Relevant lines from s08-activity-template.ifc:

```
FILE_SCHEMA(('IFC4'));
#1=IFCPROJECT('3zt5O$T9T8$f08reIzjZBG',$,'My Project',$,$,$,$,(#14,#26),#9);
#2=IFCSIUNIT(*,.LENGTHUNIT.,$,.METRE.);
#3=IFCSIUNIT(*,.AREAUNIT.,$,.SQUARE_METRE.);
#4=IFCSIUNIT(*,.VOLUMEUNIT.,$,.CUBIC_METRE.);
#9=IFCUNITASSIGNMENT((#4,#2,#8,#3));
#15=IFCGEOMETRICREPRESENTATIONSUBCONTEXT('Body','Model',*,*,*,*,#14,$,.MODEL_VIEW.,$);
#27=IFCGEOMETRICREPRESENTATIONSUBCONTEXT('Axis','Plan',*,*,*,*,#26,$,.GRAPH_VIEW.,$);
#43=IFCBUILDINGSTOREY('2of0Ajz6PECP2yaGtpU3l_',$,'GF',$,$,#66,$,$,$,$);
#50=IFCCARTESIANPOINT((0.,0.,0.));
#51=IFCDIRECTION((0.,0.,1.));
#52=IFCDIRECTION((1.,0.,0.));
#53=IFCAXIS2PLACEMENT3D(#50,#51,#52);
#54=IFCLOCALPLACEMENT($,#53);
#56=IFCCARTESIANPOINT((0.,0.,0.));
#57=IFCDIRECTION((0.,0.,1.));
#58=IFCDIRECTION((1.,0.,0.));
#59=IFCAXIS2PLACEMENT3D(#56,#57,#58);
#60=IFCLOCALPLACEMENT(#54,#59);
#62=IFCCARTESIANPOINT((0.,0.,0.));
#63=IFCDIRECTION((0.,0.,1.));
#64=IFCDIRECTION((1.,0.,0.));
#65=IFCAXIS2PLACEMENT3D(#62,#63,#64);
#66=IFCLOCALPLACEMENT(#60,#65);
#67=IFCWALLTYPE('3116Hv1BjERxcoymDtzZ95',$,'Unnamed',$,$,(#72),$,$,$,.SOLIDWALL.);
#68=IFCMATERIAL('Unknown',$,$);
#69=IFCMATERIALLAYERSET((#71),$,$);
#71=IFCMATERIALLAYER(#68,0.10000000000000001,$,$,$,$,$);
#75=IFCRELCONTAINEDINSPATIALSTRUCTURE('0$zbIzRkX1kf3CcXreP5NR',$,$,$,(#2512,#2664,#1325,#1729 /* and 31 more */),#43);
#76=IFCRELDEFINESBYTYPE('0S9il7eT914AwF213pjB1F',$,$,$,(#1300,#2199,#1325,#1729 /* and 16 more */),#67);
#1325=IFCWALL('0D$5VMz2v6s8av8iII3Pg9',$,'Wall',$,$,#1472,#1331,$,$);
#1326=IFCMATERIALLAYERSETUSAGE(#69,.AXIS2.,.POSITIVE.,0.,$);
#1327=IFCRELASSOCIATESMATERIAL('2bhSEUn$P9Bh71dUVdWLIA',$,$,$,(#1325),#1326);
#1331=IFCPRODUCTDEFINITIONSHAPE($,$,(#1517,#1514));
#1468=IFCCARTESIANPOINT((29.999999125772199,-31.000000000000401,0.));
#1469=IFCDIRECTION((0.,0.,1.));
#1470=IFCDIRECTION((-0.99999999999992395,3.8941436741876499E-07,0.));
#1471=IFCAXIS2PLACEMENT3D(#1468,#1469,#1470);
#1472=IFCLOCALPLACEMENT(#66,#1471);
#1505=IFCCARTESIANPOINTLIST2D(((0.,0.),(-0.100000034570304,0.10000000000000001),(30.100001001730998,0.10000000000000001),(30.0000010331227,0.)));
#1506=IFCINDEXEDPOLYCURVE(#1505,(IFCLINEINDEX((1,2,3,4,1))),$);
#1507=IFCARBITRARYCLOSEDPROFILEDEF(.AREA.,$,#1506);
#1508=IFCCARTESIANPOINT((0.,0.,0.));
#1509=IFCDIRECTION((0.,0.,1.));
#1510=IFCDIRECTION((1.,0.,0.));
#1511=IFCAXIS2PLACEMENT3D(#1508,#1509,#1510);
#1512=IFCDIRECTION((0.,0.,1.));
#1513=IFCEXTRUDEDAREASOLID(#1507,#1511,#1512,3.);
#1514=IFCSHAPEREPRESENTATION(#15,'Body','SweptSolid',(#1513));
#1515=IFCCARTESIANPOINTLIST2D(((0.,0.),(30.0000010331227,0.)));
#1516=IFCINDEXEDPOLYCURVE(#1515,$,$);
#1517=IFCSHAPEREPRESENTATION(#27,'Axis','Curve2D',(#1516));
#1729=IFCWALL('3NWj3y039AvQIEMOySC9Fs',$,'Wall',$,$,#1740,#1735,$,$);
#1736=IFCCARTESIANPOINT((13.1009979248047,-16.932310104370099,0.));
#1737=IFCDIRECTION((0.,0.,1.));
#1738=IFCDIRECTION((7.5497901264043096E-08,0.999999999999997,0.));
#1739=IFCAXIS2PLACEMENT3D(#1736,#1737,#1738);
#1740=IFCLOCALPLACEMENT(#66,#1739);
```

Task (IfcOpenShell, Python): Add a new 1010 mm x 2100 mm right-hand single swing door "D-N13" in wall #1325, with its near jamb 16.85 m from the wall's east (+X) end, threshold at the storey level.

```python
import numpy as np
import ifcopenshell
import ifcopenshell.api.feature
import ifcopenshell.api.geometry
import ifcopenshell.api.root
import ifcopenshell.api.spatial
import ifcopenshell.geom
import ifcopenshell.util.element
import ifcopenshell.util.placement
import ifcopenshell.util.representation
import ifcopenshell.util.shape
import ifcopenshell.util.unit

model = ifcopenshell.open("s08-activity-template.ifc")
unit_scale = ifcopenshell.util.unit.calculate_unit_scale(model)
settings = ifcopenshell.geom.settings()


def volume(element):
    """Net volume in cubic metres, openings subtracted."""
    shape = ifcopenshell.geom.create_shape(settings, element)
    return ifcopenshell.util.shape.get_volume(shape.geometry)


wall = model.by_guid("0D$5VMz2v6s8av8iII3Pg9")
storey = ifcopenshell.util.element.get_container(wall, ifc_class="IfcBuildingStorey")
context = ifcopenshell.util.representation.get_context(model, "Model", "Body", "MODEL_VIEW")
before = volume(wall)

width, height, from_end, sill = 1.01, 2.1, 16.85, 0.0  # metres

# The wall runs along its own X axis, and the end named is its -X end.
wall_shape = ifcopenshell.geom.create_shape(settings, wall)
x, y, z = ifcopenshell.util.shape.get_vertices(wall_shape.geometry).T
start = x.min() + from_end
face, thickness = float(y.min()), float(y.max() - y.min())
wall_matrix = ifcopenshell.util.placement.get_local_placement(wall.ObjectPlacement)
level = ifcopenshell.util.placement.get_local_placement(storey.ObjectPlacement)[2, 3]


def in_wall(x, y):
    """Placement at x, y metres in the wall's axes, at sill height."""
    matrix = wall_matrix.copy()
    matrix[:, 3] = wall_matrix @ np.array([x / unit_scale, y / unit_scale, 0.0, 1.0])
    matrix[2, 3] = level + sill / unit_scale
    return matrix


# Opening: a box that overshoots both wall faces by 50 mm.
opening = ifcopenshell.api.root.create_entity(model, ifc_class="IfcOpeningElement", predefined_type="OPENING")
box = ifcopenshell.api.geometry.add_wall_representation(
    model, context=context, length=width, height=height, thickness=thickness + 0.1
)
ifcopenshell.api.geometry.assign_representation(model, product=opening, representation=box)
ifcopenshell.api.geometry.edit_object_placement(model, product=opening, matrix=in_wall(start, face - 0.05), is_si=False)
ifcopenshell.api.feature.add_feature(model, feature=opening, element=wall)

door = ifcopenshell.api.root.create_entity(model, ifc_class="IfcDoor", name="D-N13", predefined_type="DOOR")
door.OverallWidth, door.OverallHeight = width / unit_scale, height / unit_scale
door.OperationType = "SINGLE_SWING_RIGHT"
body = ifcopenshell.api.geometry.add_door_representation(
    model,
    context=context,
    overall_width=door.OverallWidth,
    overall_height=door.OverallHeight,
    operation_type="SINGLE_SWING_RIGHT",
    lining_properties={"LiningDepth": thickness / unit_scale, "ThresholdDepth": thickness / unit_scale},
)
ifcopenshell.api.geometry.assign_representation(model, product=door, representation=body)
ifcopenshell.api.spatial.assign_container(model, products=[door], relating_structure=storey)
ifcopenshell.api.feature.add_filling(model, opening=opening, element=door)

# The lining spans the wall, so the door starts at the wall face.
ifcopenshell.api.geometry.edit_object_placement(model, product=door, matrix=in_wall(start, face), is_si=False)

after = volume(wall)

print(f"wall volume {before:.3f} -> {after:.3f} m3")

model.write("s08-activity-template_v2.ifc")
```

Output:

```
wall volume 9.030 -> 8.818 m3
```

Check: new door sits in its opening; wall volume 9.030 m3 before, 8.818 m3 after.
